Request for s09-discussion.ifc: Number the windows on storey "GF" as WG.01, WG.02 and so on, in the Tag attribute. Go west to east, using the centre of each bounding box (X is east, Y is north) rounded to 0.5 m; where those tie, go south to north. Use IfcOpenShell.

First a look at what the model holds.

```python
import ifcopenshell
import ifcopenshell.util.element
import ifcopenshell.util.placement

model = ifcopenshell.open("s09-discussion.ifc")
print(model.schema)
storey = next(s for s in model.by_type("IfcBuildingStorey") if s.Name == "GF")
windows = [e for e in ifcopenshell.util.element.get_decomposition(storey) if e.is_a("IfcWindow")]
for e in sorted(windows, key=lambda e: e.id()):
    origin = ifcopenshell.util.placement.get_local_placement(e.ObjectPlacement)[:3, 3]
    print(e.id(), e.Tag, e.Name, origin.round(2) + 0.0, sep=" | ")
```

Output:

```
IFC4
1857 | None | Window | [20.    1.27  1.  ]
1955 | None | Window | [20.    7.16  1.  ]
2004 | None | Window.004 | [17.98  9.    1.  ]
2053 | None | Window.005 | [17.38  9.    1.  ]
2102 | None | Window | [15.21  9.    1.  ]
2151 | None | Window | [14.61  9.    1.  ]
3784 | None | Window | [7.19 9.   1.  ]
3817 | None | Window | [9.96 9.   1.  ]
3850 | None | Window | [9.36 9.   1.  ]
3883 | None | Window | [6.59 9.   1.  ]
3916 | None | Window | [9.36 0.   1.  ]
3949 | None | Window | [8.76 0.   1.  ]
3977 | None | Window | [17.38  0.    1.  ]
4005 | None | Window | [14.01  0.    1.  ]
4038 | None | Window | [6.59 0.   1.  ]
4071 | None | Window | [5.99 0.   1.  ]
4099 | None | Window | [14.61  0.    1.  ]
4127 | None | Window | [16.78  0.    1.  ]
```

```python
import ifcopenshell
import ifcopenshell.geom
import ifcopenshell.util.element
import ifcopenshell.util.shape

model = ifcopenshell.open("s09-discussion.ifc")
settings = ifcopenshell.geom.settings()
settings.set("use-world-coords", True)


def centre(element):
    shape = ifcopenshell.geom.create_shape(settings, element)
    return ifcopenshell.util.shape.get_bbox_centroid(shape.geometry)


storey = next(s for s in model.by_type("IfcBuildingStorey") if s.Name == "GF")
windows = [e for e in ifcopenshell.util.element.get_decomposition(storey) if e.is_a("IfcWindow")]

# Insertion points can sit at a corner or the storey origin, so sort by the geometry (in metres).
centres = {e: centre(e) for e in windows}
windows.sort(key=lambda e: (round(centres[e][0] / 0.5), centres[e][1]))

for i, e in enumerate(windows, start=1):
    number = f"WG.{i:02d}"
    e.Tag = number
    print(e.id(), number)

model.write("s09-discussion_rev.ifc")
```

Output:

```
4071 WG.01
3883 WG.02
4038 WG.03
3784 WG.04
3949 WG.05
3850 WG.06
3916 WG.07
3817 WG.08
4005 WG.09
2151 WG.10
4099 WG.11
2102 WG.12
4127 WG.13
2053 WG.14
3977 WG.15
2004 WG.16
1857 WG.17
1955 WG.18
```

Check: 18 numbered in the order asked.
